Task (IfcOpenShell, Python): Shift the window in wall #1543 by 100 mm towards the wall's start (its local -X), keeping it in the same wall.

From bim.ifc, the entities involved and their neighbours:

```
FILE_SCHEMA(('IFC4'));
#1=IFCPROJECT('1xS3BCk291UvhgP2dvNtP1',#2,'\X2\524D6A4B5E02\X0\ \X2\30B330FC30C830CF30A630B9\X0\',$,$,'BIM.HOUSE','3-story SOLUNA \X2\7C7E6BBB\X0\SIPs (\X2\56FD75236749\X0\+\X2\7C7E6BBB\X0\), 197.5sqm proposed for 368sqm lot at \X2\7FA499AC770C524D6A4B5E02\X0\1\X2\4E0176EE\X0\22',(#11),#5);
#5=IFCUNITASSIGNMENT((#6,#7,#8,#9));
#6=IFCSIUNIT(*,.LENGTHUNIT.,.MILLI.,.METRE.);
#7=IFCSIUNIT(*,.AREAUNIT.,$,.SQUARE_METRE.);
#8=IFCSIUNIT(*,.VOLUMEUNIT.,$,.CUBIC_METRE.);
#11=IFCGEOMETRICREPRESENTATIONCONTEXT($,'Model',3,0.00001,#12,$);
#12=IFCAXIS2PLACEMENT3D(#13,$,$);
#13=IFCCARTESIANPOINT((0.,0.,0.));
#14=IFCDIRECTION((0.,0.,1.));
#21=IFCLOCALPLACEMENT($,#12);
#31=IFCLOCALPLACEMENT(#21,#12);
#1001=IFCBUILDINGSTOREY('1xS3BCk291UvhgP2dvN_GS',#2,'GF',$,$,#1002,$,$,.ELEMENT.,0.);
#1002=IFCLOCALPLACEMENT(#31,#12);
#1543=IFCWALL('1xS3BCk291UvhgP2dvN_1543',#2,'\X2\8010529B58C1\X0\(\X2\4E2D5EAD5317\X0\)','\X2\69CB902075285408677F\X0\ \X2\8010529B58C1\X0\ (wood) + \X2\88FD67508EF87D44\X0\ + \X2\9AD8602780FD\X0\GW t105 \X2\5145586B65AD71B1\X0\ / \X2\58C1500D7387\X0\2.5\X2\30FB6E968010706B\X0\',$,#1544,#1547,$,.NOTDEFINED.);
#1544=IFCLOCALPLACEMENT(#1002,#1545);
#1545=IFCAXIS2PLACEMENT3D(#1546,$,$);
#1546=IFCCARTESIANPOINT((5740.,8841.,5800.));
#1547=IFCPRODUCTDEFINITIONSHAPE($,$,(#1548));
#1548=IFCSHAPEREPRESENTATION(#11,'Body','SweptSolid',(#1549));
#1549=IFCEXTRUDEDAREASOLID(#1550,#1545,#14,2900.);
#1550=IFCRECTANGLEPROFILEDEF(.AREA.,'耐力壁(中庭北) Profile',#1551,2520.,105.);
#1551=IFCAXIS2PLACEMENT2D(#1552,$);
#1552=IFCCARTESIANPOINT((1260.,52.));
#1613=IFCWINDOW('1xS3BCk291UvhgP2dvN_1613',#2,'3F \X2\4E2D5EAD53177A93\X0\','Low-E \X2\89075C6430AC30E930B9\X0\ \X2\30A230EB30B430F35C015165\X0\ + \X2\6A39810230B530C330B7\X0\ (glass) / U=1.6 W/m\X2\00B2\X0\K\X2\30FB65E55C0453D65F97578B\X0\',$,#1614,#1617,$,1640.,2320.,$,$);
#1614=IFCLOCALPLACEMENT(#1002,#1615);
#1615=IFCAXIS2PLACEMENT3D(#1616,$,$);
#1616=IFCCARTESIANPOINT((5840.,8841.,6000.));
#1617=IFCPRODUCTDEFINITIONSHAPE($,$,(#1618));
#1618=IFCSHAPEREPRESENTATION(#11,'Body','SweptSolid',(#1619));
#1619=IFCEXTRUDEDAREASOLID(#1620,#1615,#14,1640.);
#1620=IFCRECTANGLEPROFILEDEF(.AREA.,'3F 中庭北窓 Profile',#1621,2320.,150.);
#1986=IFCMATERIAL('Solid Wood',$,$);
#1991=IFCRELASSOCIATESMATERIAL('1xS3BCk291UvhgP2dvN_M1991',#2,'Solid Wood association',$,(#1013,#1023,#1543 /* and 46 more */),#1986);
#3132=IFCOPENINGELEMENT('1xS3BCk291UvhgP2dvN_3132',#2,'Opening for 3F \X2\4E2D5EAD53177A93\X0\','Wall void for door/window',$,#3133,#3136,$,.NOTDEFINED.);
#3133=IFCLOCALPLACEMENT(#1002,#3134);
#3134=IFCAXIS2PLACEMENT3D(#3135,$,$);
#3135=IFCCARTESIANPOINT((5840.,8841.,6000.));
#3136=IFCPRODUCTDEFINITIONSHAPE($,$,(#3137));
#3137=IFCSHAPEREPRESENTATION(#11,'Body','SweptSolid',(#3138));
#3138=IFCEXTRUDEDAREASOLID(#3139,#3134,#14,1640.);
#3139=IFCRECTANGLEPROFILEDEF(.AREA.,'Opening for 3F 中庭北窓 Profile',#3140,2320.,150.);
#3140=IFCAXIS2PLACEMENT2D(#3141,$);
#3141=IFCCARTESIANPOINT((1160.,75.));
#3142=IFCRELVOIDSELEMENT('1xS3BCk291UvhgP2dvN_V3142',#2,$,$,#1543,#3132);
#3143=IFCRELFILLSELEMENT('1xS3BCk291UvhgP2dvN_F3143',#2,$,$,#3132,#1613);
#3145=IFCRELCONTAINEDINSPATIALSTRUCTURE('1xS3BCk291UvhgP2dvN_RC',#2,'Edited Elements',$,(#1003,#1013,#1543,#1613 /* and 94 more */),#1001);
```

```python
import ifcopenshell
import ifcopenshell.api.geometry
import ifcopenshell.util.placement
import ifcopenshell.util.unit

model = ifcopenshell.open("bim.ifc")
unit_scale = ifcopenshell.util.unit.calculate_unit_scale(model)

window = model.by_guid("1xS3BCk291UvhgP2dvN_1613")
opening = window.FillsVoids[0].RelatingOpeningElement
wall = opening.VoidsElements[0].RelatingBuildingElement

wall_matrix = ifcopenshell.util.placement.get_local_placement(wall.ObjectPlacement)
shift = wall_matrix[:3, 0] * -0.1 / unit_scale
before = ifcopenshell.util.placement.get_local_placement(window.ObjectPlacement)[:3, 3].copy()

# The window is not placed relative to its opening, so move both.
for product in (opening, window):
    matrix = ifcopenshell.util.placement.get_local_placement(product.ObjectPlacement)
    matrix[:3, 3] += shift
    ifcopenshell.api.geometry.edit_object_placement(model, product=product, matrix=matrix, is_si=False)

after = ifcopenshell.util.placement.get_local_placement(window.ObjectPlacement)[:3, 3]
print("window moved by", (after - before).round(3) + 0.0)

model.write("bim_rev.ifc")
```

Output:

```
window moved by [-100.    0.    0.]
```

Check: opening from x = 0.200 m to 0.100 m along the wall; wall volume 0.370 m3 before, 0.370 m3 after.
